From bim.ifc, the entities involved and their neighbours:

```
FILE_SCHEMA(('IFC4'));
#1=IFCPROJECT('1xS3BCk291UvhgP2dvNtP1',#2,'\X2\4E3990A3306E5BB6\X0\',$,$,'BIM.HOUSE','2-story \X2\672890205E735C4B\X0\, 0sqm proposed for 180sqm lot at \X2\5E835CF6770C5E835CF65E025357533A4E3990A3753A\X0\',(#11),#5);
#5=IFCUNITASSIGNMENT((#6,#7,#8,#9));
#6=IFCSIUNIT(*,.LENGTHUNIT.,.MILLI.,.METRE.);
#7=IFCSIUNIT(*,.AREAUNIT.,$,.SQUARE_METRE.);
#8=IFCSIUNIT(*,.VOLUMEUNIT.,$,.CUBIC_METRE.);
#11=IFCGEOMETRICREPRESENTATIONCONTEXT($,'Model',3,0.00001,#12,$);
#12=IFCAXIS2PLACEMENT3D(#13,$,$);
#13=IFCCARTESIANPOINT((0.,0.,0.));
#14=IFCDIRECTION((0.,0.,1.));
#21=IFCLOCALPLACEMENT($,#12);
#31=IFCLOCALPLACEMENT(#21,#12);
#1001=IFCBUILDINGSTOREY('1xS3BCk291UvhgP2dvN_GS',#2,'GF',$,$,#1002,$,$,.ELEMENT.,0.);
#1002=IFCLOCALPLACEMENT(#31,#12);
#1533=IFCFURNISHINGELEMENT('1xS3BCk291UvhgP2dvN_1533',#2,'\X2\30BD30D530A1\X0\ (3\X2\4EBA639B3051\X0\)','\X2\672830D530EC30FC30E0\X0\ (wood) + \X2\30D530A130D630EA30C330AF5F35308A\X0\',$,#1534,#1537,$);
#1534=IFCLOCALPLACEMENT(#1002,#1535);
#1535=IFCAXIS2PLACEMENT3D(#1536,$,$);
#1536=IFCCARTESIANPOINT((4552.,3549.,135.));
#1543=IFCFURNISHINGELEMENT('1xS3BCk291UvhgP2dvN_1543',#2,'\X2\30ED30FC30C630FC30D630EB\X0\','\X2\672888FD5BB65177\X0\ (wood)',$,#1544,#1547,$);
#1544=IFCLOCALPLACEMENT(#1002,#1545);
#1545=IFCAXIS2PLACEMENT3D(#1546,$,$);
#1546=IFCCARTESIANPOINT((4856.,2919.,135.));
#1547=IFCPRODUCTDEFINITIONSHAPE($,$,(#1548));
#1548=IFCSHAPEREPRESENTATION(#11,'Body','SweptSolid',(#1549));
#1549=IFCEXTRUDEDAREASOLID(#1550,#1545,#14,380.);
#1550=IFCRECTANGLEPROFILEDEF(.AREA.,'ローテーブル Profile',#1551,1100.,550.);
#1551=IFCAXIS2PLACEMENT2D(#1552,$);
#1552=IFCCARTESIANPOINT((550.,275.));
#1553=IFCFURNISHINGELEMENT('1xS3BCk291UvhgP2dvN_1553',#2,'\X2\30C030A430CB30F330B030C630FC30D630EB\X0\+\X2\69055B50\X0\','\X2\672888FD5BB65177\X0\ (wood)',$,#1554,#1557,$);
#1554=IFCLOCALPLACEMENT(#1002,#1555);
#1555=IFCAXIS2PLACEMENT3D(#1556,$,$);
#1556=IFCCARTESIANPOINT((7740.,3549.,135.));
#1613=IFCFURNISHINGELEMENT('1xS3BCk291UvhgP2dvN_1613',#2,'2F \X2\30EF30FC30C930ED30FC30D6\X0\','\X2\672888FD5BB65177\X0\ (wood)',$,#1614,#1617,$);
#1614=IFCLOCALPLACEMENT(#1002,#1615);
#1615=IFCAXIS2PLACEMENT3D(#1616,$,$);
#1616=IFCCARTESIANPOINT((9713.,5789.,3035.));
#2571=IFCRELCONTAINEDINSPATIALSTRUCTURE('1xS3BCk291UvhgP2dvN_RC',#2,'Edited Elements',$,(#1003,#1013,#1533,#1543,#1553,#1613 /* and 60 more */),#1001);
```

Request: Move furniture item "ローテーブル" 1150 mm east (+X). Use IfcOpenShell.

```python
import ifcopenshell
import ifcopenshell.api.geometry
import ifcopenshell.util.placement
import ifcopenshell.util.unit

model = ifcopenshell.open("bim.ifc")
unit_scale = ifcopenshell.util.unit.calculate_unit_scale(model)

item = model.by_guid("1xS3BCk291UvhgP2dvN_1543")
matrix = ifcopenshell.util.placement.get_local_placement(item.ObjectPlacement)
matrix[0, 3] += 1.15 / unit_scale
ifcopenshell.api.geometry.edit_object_placement(model, product=item, matrix=matrix, is_si=False)

print(ifcopenshell.util.placement.get_local_placement(item.ObjectPlacement).round(3) + 0.0)

model.write("bim_edited.ifc")
```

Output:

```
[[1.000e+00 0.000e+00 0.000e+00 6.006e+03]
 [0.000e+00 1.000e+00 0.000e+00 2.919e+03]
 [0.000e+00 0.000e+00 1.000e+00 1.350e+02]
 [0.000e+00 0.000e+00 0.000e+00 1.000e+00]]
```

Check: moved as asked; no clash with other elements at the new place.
